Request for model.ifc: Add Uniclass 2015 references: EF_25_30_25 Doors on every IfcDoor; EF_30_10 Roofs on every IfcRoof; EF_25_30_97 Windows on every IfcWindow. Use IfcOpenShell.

First a look at what the model holds.

```python
import ifcopenshell

model = ifcopenshell.open("model.ifc")
print(model.schema)
print("classifications:", [c.Name for c in model.by_type("IfcClassification")])
for ifc_class in ("IfcDoor", "IfcRoof", "IfcStair", "IfcWall", "IfcWindow"):
    print(ifc_class, len(model.by_type(ifc_class)))
```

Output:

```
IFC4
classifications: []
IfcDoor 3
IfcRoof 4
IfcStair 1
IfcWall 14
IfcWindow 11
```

```python
import ifcopenshell
import ifcopenshell.api.classification

model = ifcopenshell.open("model.ifc")

system = ifcopenshell.api.classification.add_classification(model, classification="Uniclass 2015")

codes = {
    "IfcDoor": ("EF_25_30_25", "Doors"),
    "IfcRoof": ("EF_30_10", "Roofs"),
    "IfcWindow": ("EF_25_30_97", "Windows"),
}
for ifc_class, (code, name) in codes.items():
    products = model.by_type(ifc_class)
    ifcopenshell.api.classification.add_reference(
        model, products=products, classification=system, identification=code, name=name
    )
    print(code, len(products))

model.write("model-out.ifc")
```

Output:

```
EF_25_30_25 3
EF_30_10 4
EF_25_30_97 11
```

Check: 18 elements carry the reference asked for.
